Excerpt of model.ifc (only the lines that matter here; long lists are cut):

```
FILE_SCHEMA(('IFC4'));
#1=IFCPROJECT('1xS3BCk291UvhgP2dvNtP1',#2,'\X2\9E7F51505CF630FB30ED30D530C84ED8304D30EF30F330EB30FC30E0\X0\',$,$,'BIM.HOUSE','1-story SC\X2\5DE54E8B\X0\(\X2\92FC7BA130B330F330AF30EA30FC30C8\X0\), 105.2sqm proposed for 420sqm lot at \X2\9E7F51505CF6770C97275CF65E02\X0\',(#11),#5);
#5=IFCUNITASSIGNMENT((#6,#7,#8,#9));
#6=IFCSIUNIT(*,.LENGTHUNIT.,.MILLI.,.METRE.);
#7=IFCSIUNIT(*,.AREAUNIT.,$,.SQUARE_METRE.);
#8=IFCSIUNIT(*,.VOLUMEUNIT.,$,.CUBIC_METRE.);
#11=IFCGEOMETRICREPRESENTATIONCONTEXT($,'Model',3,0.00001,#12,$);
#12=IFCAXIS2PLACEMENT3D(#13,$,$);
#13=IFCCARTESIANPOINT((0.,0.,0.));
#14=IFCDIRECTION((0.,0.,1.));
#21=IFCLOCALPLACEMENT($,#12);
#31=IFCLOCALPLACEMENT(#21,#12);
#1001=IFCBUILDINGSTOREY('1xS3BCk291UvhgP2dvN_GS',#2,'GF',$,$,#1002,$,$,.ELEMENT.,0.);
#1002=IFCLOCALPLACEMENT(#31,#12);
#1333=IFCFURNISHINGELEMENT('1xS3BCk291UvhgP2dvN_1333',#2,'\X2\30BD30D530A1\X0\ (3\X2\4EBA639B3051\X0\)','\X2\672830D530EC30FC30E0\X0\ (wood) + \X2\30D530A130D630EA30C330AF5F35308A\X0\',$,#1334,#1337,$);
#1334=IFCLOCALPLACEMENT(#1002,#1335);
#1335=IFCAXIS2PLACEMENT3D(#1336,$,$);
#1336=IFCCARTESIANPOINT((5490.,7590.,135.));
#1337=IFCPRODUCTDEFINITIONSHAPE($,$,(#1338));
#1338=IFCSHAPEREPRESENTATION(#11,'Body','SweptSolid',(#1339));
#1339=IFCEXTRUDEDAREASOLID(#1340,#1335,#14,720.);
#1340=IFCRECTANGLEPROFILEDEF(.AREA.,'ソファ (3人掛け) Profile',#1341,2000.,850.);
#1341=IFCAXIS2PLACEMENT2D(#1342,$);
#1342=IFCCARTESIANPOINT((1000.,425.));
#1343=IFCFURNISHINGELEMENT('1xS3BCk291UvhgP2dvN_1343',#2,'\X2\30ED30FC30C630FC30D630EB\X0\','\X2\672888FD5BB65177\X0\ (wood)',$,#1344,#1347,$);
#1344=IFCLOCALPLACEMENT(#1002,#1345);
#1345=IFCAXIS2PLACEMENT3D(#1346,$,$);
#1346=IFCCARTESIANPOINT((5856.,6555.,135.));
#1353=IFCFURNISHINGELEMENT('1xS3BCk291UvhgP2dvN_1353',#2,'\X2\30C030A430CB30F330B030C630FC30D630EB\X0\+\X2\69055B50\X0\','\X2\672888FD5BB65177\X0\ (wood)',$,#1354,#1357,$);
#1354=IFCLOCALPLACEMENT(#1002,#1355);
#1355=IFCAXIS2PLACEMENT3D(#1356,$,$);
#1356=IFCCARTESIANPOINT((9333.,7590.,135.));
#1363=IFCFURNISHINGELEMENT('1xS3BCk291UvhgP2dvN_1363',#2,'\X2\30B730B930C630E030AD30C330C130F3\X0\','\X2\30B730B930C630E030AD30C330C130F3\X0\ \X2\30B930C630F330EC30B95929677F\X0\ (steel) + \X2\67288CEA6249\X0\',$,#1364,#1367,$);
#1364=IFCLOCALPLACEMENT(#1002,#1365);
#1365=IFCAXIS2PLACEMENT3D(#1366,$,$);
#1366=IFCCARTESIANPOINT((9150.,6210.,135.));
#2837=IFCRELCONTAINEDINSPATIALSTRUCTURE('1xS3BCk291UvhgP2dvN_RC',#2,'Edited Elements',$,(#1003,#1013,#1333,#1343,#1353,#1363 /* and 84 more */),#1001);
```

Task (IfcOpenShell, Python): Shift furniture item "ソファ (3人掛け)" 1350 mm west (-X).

```python
import ifcopenshell
import ifcopenshell.api.geometry
import ifcopenshell.util.placement
import ifcopenshell.util.unit

model = ifcopenshell.open("model.ifc")
unit_scale = ifcopenshell.util.unit.calculate_unit_scale(model)

item = model.by_guid("1xS3BCk291UvhgP2dvN_1333")
matrix = ifcopenshell.util.placement.get_local_placement(item.ObjectPlacement)
matrix[0, 3] -= 1.35 / unit_scale
ifcopenshell.api.geometry.edit_object_placement(model, product=item, matrix=matrix, is_si=False)

print(ifcopenshell.util.placement.get_local_placement(item.ObjectPlacement).round(3) + 0.0)

model.write("model_v2.ifc")
```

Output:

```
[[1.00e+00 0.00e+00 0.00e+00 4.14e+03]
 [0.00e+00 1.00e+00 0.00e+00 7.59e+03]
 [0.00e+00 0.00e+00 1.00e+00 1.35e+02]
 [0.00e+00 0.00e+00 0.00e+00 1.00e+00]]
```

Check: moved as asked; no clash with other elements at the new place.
